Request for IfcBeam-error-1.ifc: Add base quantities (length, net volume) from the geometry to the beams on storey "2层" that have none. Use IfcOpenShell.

First a look at what the model holds.

```python
import ifcopenshell
import ifcopenshell.util.element
import ifcopenshell.util.unit

model = ifcopenshell.open("IfcBeam-error-1.ifc")
print(model.schema)
for unit_type in ("LENGTHUNIT", "AREAUNIT", "VOLUMEUNIT"):
    print(unit_type, ifcopenshell.util.unit.calculate_unit_scale(model, unit_type))
storey = next(s for s in model.by_type("IfcBuildingStorey") if s.Name == "2层")
beams = [e for e in ifcopenshell.util.element.get_decomposition(storey) if e.is_a("IfcBeam")]
for e in sorted(beams, key=lambda e: e.id()):
    print(e.id(), e.is_a(), e.Name, list(ifcopenshell.util.element.get_psets(e, qtos_only=True)), sep=" | ")
```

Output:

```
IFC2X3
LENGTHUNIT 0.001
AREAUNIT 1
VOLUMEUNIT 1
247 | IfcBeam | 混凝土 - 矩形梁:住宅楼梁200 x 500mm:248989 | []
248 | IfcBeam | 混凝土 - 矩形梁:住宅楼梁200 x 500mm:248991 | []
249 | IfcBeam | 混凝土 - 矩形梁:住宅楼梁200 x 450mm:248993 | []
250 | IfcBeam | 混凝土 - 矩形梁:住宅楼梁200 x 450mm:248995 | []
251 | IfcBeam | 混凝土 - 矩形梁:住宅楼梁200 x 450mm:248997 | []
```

```python
import ifcopenshell
import ifcopenshell.api.pset
import ifcopenshell.geom
import ifcopenshell.util.element
import ifcopenshell.util.shape
import ifcopenshell.util.unit

model = ifcopenshell.open("IfcBeam-error-1.ifc")
unit_scale = ifcopenshell.util.unit.calculate_unit_scale(model)
volume_scale = ifcopenshell.util.unit.calculate_unit_scale(model, "VOLUMEUNIT")
settings = ifcopenshell.geom.settings()

storey = next(s for s in model.by_type("IfcBuildingStorey") if s.Name == "2层")
beams = [e for e in ifcopenshell.util.element.get_decomposition(storey) if e.is_a("IfcBeam")]

for e in sorted(beams, key=lambda e: e.id()):
    if ifcopenshell.util.element.get_psets(e, qtos_only=True, should_inherit=False):
        continue
    # Geometry comes back in metres, in the element's own axes.
    shape = ifcopenshell.geom.create_shape(settings, e)
    values = {
        "Length": ifcopenshell.util.shape.get_max_xyz(shape.geometry) / unit_scale,
        "NetVolume": ifcopenshell.util.shape.get_volume(shape.geometry) / volume_scale,
    }
    qto = ifcopenshell.api.pset.add_qto(model, product=e, name="BaseQuantities")
    ifcopenshell.api.pset.edit_qto(model, qto=qto, properties=values)
    print(e.id(), {k: round(v, 3) for k, v in values.items()})

model.write("IfcBeam-error-1-out.ifc")
```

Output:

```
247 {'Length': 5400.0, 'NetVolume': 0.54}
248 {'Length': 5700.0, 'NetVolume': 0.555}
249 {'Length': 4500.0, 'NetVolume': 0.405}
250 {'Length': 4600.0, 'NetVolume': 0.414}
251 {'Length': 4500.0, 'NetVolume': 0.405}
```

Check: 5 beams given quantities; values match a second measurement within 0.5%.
